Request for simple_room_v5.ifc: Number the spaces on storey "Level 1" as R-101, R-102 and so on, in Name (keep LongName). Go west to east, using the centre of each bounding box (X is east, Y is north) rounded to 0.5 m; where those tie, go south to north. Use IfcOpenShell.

First a look at what the model holds.

```python
import ifcopenshell
import ifcopenshell.util.element
import ifcopenshell.util.placement

model = ifcopenshell.open("simple_room_v5.ifc")
print(model.schema)
storey = next(s for s in model.by_type("IfcBuildingStorey") if s.Name == "Level 1")
spaces = [e for e in ifcopenshell.util.element.get_decomposition(storey) if e.is_a("IfcSpace")]
for e in sorted(spaces, key=lambda e: e.id()):
    origin = ifcopenshell.util.placement.get_local_placement(e.ObjectPlacement)[:3, 3]
    print(e.id(), e.Name, e.LongName, origin.round(2) + 0.0, sep=" | ")
```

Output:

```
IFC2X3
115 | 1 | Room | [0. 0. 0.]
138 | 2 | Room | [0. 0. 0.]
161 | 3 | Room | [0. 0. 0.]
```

```python
import ifcopenshell
import ifcopenshell.geom
import ifcopenshell.util.element
import ifcopenshell.util.shape

model = ifcopenshell.open("simple_room_v5.ifc")
settings = ifcopenshell.geom.settings()
settings.set("use-world-coords", True)


def centre(element):
    shape = ifcopenshell.geom.create_shape(settings, element)
    return ifcopenshell.util.shape.get_bbox_centroid(shape.geometry)


storey = next(s for s in model.by_type("IfcBuildingStorey") if s.Name == "Level 1")
spaces = [e for e in ifcopenshell.util.element.get_decomposition(storey) if e.is_a("IfcSpace")]

# Insertion points can sit at a corner or the storey origin, so sort by the geometry (in metres).
centres = {e: centre(e) for e in spaces}
spaces.sort(key=lambda e: (round(centres[e][0] / 0.5), centres[e][1]))

for i, e in enumerate(spaces, start=1):
    number = f"R-1{i:02d}"
    e.Name = number
    print(e.id(), number)

model.write("simple_room_v5-out.ifc")
```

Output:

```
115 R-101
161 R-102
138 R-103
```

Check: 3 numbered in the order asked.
